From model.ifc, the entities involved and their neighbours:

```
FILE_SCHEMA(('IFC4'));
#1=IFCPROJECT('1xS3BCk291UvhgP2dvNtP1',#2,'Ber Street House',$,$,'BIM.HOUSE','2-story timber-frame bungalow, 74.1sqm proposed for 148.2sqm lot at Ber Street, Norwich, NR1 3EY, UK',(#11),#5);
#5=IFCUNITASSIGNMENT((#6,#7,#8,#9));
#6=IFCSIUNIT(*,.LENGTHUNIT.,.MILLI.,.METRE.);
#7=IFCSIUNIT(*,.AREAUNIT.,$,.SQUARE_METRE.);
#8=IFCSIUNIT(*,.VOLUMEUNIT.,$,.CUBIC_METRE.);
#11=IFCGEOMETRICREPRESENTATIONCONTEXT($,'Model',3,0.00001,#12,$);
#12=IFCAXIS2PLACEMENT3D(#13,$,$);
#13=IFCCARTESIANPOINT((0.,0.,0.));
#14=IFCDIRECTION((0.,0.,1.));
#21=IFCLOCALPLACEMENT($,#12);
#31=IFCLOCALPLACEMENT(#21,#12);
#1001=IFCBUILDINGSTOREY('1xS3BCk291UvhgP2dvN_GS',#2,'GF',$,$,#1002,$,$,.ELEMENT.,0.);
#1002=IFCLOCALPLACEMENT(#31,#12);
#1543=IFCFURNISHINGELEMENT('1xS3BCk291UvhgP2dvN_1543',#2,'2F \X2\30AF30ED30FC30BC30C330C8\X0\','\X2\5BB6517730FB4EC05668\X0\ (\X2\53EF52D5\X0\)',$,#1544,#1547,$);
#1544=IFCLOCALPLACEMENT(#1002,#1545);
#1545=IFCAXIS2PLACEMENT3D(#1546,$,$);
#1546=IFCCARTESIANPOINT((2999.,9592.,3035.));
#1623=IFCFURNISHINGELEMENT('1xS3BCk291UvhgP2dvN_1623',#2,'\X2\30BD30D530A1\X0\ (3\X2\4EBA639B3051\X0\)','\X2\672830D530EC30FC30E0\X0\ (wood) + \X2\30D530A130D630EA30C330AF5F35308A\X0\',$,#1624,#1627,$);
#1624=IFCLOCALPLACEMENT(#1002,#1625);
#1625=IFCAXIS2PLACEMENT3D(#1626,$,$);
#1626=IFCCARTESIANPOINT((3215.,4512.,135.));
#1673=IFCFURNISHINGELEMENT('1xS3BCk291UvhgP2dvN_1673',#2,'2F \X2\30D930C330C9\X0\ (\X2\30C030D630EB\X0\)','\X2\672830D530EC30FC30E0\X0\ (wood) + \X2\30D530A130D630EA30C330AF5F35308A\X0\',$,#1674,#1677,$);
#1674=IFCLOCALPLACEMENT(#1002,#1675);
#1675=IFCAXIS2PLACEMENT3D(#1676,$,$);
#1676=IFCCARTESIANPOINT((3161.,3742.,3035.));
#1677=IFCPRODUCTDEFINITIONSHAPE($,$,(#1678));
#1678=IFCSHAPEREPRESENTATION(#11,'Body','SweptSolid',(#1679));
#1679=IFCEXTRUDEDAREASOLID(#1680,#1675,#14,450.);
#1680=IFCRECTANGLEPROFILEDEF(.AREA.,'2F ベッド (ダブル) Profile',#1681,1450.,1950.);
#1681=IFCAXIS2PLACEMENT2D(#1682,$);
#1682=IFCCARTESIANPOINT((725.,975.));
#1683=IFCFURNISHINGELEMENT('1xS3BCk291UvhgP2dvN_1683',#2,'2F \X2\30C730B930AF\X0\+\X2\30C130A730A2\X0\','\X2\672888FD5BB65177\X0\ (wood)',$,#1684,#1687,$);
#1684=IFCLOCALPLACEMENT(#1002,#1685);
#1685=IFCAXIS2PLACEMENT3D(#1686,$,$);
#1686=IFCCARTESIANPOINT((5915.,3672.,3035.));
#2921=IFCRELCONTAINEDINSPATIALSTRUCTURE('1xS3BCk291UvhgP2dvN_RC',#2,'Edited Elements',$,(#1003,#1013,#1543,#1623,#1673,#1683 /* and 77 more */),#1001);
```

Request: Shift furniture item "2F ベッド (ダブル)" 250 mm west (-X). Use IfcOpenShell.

```python
import ifcopenshell
import ifcopenshell.api.geometry
import ifcopenshell.util.placement
import ifcopenshell.util.unit

model = ifcopenshell.open("model.ifc")
unit_scale = ifcopenshell.util.unit.calculate_unit_scale(model)

item = model.by_id(1673)
matrix = ifcopenshell.util.placement.get_local_placement(item.ObjectPlacement)
matrix[0, 3] -= 0.25 / unit_scale
ifcopenshell.api.geometry.edit_object_placement(model, product=item, matrix=matrix, is_si=False)

print(ifcopenshell.util.placement.get_local_placement(item.ObjectPlacement).round(3) + 0.0)

model.write("model_rev.ifc")
```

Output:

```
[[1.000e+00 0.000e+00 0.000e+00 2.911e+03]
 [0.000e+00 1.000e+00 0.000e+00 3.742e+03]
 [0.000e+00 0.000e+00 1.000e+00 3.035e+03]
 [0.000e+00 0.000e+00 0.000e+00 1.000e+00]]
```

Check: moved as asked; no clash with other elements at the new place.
